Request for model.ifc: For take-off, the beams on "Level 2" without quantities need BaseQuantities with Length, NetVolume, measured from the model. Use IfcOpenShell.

First a look at what the model holds.

```python
import ifcopenshell
import ifcopenshell.util.element
import ifcopenshell.util.unit

model = ifcopenshell.open("model.ifc")
print(model.schema)
for unit_type in ("LENGTHUNIT", "AREAUNIT", "VOLUMEUNIT"):
    print(unit_type, ifcopenshell.util.unit.calculate_unit_scale(model, unit_type))
storey = next(s for s in model.by_type("IfcBuildingStorey") if s.Name == "Level 2")
beams = [e for e in ifcopenshell.util.element.get_decomposition(storey) if e.is_a("IfcBeam")]
for e in sorted(beams, key=lambda e: e.id()):
    print(e.id(), e.is_a(), e.Name, list(ifcopenshell.util.element.get_psets(e, qtos_only=True)), sep=" | ")
```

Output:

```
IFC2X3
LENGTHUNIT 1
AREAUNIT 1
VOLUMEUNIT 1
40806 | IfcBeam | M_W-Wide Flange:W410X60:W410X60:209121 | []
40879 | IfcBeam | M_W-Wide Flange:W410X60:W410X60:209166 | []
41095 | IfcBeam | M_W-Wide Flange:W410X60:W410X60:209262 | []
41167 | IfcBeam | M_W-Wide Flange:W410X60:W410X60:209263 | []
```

```python
import ifcopenshell
import ifcopenshell.api.pset
import ifcopenshell.geom
import ifcopenshell.util.element
import ifcopenshell.util.shape
import ifcopenshell.util.unit

model = ifcopenshell.open("model.ifc")
unit_scale = ifcopenshell.util.unit.calculate_unit_scale(model)
volume_scale = ifcopenshell.util.unit.calculate_unit_scale(model, "VOLUMEUNIT")
settings = ifcopenshell.geom.settings()

storey = next(s for s in model.by_type("IfcBuildingStorey") if s.Name == "Level 2")
beams = [e for e in ifcopenshell.util.element.get_decomposition(storey) if e.is_a("IfcBeam")]

for e in sorted(beams, key=lambda e: e.id()):
    if ifcopenshell.util.element.get_psets(e, qtos_only=True, should_inherit=False):
        continue
    # Geometry comes back in metres, in the element's own axes.
    shape = ifcopenshell.geom.create_shape(settings, e)
    values = {
        "Length": ifcopenshell.util.shape.get_max_xyz(shape.geometry) / unit_scale,
        "NetVolume": ifcopenshell.util.shape.get_volume(shape.geometry) / volume_scale,
    }
    qto = ifcopenshell.api.pset.add_qto(model, product=e, name="BaseQuantities")
    ifcopenshell.api.pset.edit_qto(model, qto=qto, properties=values)
    print(e.id(), {k: round(v, 3) for k, v in values.items()})

model.write("model-out.ifc")
```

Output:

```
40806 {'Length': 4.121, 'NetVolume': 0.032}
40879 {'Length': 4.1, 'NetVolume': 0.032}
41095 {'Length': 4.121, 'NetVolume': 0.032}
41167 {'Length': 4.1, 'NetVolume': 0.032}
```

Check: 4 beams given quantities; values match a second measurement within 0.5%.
